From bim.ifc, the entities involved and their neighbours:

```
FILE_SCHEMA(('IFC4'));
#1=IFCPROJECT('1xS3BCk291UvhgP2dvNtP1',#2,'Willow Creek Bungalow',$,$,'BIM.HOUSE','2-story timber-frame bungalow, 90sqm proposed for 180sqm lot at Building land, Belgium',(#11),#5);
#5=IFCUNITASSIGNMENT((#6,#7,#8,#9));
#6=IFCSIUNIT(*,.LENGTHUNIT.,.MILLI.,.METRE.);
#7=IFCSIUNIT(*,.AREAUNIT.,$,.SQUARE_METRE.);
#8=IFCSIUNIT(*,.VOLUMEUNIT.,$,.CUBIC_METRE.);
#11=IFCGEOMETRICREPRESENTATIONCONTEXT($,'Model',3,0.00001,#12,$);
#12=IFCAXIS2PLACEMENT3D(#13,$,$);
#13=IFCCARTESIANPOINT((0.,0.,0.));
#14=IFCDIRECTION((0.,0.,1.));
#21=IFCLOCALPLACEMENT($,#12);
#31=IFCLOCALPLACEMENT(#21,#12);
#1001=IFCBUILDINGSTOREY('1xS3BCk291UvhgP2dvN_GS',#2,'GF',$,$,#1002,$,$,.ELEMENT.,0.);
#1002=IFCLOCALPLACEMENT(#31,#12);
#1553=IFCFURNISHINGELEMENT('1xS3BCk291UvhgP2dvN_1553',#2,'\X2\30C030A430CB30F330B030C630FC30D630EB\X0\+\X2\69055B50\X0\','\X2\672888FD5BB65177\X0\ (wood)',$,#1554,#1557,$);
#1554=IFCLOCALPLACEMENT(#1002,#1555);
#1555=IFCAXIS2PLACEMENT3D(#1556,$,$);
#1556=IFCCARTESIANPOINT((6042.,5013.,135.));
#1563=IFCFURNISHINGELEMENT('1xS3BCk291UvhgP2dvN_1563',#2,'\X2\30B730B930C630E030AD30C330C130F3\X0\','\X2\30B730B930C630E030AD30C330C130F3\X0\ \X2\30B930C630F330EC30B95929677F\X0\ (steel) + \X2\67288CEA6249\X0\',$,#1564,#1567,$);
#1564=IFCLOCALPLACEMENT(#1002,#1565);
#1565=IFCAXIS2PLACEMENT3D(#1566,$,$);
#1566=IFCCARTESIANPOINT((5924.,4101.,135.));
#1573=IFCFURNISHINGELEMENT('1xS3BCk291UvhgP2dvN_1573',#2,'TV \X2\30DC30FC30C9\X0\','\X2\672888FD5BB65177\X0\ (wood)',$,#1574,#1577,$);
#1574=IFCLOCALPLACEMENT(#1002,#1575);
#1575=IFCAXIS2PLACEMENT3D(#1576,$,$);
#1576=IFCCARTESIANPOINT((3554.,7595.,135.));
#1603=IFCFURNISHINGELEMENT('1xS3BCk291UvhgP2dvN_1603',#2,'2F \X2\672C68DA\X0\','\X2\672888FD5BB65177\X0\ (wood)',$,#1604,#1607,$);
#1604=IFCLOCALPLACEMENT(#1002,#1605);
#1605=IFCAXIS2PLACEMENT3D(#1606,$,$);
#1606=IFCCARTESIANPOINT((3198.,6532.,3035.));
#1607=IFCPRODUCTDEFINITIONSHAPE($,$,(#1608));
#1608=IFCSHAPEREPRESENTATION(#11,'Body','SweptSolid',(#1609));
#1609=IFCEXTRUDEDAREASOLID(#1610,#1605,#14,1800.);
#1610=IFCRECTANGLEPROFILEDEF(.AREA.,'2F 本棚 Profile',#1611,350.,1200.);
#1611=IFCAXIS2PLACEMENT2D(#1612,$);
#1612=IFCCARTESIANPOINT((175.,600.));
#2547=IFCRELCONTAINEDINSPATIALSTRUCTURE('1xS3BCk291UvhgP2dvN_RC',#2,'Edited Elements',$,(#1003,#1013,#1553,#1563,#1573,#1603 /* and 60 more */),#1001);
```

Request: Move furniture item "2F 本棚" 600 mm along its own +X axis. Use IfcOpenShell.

```python
import ifcopenshell
import ifcopenshell.api.geometry
import ifcopenshell.util.placement
import ifcopenshell.util.unit

model = ifcopenshell.open("bim.ifc")
unit_scale = ifcopenshell.util.unit.calculate_unit_scale(model)

item = model.by_guid("1xS3BCk291UvhgP2dvN_1603")
matrix = ifcopenshell.util.placement.get_local_placement(item.ObjectPlacement)
matrix[:3, 3] += matrix[:3, 0] * 0.6 / unit_scale
ifcopenshell.api.geometry.edit_object_placement(model, product=item, matrix=matrix, is_si=False)

print(ifcopenshell.util.placement.get_local_placement(item.ObjectPlacement).round(3) + 0.0)

model.write("bim_edited.ifc")
```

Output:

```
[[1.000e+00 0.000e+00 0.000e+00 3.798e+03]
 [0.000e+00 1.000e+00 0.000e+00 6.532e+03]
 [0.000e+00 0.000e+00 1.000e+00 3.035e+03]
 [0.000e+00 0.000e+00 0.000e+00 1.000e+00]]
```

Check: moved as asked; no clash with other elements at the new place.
